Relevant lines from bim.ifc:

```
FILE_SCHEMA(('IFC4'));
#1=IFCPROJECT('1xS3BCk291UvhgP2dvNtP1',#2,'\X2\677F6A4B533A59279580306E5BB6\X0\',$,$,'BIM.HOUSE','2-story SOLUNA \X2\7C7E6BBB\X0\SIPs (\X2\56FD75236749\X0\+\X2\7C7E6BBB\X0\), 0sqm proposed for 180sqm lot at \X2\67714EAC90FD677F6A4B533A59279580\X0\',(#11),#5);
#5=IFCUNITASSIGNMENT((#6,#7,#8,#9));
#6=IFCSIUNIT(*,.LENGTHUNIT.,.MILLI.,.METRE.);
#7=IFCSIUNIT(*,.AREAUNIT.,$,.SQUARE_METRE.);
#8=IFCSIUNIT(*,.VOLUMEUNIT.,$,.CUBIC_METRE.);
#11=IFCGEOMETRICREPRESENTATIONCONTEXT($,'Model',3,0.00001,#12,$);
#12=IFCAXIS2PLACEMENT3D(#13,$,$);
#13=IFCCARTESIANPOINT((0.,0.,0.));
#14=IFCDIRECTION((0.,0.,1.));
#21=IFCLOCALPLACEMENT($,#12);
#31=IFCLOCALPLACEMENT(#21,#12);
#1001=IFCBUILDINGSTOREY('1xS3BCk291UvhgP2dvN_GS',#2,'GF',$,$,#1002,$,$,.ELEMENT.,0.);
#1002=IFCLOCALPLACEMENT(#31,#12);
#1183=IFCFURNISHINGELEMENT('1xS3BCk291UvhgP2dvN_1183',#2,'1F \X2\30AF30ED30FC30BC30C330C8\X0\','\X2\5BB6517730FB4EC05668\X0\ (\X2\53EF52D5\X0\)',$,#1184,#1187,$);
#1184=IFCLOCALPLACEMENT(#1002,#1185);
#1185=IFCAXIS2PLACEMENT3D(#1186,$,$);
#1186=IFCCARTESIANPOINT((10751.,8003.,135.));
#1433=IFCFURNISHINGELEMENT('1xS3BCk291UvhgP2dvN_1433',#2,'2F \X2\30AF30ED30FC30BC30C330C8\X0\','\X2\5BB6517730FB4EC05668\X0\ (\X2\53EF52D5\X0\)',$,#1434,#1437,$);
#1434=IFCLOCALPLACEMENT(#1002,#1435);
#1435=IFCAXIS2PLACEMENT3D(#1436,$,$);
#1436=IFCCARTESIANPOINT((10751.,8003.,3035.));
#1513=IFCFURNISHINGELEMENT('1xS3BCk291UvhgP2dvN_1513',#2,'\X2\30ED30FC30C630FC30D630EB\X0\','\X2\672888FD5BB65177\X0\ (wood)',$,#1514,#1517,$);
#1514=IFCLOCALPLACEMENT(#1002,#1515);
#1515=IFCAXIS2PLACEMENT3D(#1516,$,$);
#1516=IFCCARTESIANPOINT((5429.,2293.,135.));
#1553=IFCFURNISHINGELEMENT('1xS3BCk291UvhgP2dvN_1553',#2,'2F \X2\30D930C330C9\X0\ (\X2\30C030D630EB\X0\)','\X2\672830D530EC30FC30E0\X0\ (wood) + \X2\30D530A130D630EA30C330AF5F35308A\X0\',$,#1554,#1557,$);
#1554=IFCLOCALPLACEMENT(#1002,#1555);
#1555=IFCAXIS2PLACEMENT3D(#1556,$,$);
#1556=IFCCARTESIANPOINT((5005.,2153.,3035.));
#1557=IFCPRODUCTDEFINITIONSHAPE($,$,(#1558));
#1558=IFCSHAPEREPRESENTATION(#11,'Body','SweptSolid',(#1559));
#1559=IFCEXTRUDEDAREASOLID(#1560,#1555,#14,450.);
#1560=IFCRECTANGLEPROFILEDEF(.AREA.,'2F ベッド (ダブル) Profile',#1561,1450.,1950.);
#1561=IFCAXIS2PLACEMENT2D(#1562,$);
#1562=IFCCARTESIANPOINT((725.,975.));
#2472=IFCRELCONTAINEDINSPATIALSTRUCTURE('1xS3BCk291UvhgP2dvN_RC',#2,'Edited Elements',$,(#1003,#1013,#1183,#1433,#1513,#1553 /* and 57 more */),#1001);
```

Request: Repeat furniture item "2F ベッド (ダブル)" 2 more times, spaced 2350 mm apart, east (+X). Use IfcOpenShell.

```python
import numpy as np
import ifcopenshell
import ifcopenshell.api.geometry
import ifcopenshell.api.root
import ifcopenshell.util.element
import ifcopenshell.util.placement
import ifcopenshell.util.unit

model = ifcopenshell.open("bim.ifc")
unit_scale = ifcopenshell.util.unit.calculate_unit_scale(model)


def reuse_history(source, copy):
    """copy_class also copies each property set's owner history, people and application; keep the originals."""
    for rel in copy.IsDefinedBy:
        if rel.is_a("IfcRelDefinesByProperties") and (history := rel.RelatingPropertyDefinition.OwnerHistory):
            rel.RelatingPropertyDefinition.OwnerHistory = source.OwnerHistory
            ifcopenshell.util.element.remove_deep2(model, history)


source = model.by_guid("1xS3BCk291UvhgP2dvN_1553")
base = ifcopenshell.util.placement.get_local_placement(source.ObjectPlacement)
step = np.array([1.0, 0.0, 0.0]) * 2.35 / unit_scale

for i in range(1, 3):
    copy = ifcopenshell.api.root.copy_class(model, product=source)
    copy.Representation = ifcopenshell.util.element.copy_deep(
        model, source.Representation, exclude=["IfcGeometricRepresentationContext", "IfcRepresentationMap"]
    )
    reuse_history(source, copy)
    matrix = base.copy()
    matrix[:3, 3] += i * step
    print("added at", matrix[:3, 3].round(3) + 0.0)
    ifcopenshell.api.geometry.edit_object_placement(model, product=copy, matrix=matrix, is_si=False)

model.write("bim_updated.ifc")
```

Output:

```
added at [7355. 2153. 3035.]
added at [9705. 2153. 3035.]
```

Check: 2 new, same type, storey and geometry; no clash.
